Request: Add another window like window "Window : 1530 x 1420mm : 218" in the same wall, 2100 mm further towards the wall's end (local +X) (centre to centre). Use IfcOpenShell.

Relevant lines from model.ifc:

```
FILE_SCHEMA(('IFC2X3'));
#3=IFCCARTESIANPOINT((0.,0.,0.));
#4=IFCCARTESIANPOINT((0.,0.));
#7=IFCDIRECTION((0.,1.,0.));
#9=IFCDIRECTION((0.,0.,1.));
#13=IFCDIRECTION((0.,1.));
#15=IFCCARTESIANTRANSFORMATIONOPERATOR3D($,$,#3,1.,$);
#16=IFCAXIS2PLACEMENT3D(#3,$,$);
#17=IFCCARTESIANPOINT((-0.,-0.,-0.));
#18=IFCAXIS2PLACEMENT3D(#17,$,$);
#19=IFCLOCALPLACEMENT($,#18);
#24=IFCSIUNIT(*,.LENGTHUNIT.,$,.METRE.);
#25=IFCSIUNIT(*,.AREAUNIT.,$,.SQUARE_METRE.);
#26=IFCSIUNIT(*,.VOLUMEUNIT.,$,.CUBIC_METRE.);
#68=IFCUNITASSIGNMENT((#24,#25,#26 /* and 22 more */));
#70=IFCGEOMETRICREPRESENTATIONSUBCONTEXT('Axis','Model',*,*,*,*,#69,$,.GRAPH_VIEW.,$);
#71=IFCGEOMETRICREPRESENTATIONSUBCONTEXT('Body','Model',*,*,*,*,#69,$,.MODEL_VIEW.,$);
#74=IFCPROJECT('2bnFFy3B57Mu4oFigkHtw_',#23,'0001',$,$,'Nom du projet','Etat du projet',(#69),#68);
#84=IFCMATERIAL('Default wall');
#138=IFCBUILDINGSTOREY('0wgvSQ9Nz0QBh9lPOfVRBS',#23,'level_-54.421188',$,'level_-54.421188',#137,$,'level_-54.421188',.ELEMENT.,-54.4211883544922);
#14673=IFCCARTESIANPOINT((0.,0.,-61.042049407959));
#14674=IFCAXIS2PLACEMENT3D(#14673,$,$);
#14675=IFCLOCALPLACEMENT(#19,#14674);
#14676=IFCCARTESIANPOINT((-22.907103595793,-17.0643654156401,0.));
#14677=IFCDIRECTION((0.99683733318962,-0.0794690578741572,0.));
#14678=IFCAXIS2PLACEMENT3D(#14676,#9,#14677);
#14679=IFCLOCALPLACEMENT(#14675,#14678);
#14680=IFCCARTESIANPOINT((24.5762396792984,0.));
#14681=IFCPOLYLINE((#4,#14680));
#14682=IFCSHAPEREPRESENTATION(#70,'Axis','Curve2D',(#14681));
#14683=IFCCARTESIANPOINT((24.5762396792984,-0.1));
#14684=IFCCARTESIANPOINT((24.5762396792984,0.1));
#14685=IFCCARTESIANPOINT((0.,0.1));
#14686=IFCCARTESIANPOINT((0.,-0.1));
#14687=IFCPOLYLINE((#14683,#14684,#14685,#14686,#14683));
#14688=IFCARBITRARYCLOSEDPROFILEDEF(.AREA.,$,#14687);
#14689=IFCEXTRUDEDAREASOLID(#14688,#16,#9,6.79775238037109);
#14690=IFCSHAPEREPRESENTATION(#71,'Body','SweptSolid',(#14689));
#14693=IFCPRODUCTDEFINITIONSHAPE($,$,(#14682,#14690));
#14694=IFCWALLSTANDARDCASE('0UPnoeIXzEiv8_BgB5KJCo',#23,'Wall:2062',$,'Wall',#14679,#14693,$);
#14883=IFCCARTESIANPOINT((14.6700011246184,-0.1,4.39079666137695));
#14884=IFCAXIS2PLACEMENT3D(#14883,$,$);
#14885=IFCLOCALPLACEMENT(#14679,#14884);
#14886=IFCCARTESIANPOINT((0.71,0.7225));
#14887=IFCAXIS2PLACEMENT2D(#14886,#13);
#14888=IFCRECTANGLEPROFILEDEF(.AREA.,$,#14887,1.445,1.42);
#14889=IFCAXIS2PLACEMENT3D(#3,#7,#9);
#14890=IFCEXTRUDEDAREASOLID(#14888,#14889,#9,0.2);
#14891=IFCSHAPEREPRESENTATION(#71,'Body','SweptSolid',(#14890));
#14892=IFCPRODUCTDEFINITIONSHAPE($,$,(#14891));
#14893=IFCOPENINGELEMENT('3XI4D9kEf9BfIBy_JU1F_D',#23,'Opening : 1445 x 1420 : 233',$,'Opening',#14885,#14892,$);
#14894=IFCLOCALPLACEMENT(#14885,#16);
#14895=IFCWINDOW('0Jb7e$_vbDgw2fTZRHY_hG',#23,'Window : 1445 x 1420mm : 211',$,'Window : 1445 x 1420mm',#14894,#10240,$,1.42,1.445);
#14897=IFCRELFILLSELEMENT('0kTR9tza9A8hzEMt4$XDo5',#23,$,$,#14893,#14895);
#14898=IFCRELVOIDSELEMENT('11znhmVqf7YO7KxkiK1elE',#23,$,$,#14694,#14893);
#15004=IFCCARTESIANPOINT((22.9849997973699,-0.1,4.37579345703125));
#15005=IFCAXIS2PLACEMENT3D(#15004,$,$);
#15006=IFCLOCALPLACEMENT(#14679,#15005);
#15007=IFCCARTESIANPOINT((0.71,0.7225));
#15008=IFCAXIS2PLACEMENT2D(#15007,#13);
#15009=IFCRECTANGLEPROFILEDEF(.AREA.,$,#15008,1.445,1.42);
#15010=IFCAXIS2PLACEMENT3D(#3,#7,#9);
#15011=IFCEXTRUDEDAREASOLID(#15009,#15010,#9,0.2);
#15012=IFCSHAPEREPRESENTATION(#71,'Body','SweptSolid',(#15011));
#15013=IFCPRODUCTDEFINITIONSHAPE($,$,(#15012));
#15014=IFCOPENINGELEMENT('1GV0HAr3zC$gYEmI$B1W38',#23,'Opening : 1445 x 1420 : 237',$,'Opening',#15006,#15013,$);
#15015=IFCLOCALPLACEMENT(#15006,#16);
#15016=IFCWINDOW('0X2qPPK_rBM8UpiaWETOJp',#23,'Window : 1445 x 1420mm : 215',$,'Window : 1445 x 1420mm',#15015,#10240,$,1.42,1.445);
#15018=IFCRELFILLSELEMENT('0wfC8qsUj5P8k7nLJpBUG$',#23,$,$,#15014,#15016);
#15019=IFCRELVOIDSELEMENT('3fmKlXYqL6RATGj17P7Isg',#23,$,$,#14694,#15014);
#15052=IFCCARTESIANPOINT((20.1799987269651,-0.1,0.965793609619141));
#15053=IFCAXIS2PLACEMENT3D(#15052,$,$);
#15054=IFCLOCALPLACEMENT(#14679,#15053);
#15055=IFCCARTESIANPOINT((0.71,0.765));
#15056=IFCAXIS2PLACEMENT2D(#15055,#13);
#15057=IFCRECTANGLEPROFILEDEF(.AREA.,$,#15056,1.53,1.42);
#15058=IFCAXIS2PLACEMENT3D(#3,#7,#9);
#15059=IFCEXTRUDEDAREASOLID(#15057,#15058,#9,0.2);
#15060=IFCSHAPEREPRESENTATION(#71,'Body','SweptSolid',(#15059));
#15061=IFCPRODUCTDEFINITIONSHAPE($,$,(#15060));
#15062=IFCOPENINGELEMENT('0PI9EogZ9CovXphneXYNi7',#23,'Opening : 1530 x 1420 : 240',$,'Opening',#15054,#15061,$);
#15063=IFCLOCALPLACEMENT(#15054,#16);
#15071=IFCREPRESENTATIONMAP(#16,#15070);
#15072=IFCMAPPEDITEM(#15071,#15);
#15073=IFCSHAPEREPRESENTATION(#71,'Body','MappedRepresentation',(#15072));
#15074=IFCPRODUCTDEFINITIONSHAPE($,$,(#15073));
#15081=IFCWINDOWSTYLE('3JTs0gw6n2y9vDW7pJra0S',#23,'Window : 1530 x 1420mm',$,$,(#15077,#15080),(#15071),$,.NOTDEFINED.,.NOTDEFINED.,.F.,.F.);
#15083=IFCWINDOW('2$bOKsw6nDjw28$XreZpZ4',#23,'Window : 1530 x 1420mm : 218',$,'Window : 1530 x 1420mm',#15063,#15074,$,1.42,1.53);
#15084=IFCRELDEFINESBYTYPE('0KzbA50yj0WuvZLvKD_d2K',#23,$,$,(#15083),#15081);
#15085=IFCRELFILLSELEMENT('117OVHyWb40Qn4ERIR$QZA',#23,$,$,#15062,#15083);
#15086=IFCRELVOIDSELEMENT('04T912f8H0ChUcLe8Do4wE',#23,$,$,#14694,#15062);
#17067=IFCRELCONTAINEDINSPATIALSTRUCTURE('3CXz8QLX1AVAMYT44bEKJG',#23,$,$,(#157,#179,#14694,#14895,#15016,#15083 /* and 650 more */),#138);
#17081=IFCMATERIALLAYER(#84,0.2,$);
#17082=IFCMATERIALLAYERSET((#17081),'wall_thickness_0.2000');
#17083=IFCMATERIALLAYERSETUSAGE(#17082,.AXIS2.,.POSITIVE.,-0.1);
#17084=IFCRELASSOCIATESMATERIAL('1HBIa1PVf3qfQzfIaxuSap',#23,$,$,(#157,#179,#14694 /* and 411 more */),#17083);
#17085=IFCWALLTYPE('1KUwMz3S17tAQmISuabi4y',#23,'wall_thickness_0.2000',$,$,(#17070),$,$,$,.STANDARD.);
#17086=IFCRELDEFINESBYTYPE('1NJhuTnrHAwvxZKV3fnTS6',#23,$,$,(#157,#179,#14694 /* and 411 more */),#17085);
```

```python
import ifcopenshell
import ifcopenshell.api.feature
import ifcopenshell.api.geometry
import ifcopenshell.api.root
import ifcopenshell.geom
import ifcopenshell.util.element
import ifcopenshell.util.placement
import ifcopenshell.util.shape

model = ifcopenshell.open("model.ifc")
settings = ifcopenshell.geom.settings()


def volume(element):
    """Net volume in cubic metres, openings subtracted."""
    shape = ifcopenshell.geom.create_shape(settings, element)
    return ifcopenshell.util.shape.get_volume(shape.geometry)


window = model.by_guid("2$bOKsw6nDjw28$XreZpZ4")
opening = window.FillsVoids[0].RelatingOpeningElement
wall = opening.VoidsElements[0].RelatingBuildingElement
before = volume(wall)
shift = ifcopenshell.util.placement.get_local_placement(wall.ObjectPlacement)[:3, 0] * 2.1

# copy_class copies the void relationship, type, container and properties, but no geometry.
new_opening = ifcopenshell.api.root.copy_class(model, product=opening)
new_opening.Representation = ifcopenshell.util.element.copy_deep(
    model, opening.Representation, exclude=["IfcGeometricRepresentationContext", "IfcRepresentationMap"]
)
new_opening.Name = "Opening : 1530 x 1420"
new_window = ifcopenshell.api.root.copy_class(model, product=window)
new_window.Representation = ifcopenshell.util.element.copy_deep(
    model, window.Representation, exclude=["IfcGeometricRepresentationContext", "IfcRepresentationMap"]
)
new_window.Name = "Window : 1530 x 1420mm"
fills = ifcopenshell.api.feature.add_filling(model, opening=new_opening, element=new_window)
fills.OwnerHistory = new_window.OwnerHistory  # required in IFC2X3

for old, new in ((opening, new_opening), (window, new_window)):
    matrix = ifcopenshell.util.placement.get_local_placement(old.ObjectPlacement)
    matrix[:3, 3] += shift
    ifcopenshell.api.geometry.edit_object_placement(model, product=new, matrix=matrix, is_si=False)

after = volume(wall)

print(f"wall volume {before:.3f} -> {after:.3f} m3")

model.write("model_v2.ifc")
```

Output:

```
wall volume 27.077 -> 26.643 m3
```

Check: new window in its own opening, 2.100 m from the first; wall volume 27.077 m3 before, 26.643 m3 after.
